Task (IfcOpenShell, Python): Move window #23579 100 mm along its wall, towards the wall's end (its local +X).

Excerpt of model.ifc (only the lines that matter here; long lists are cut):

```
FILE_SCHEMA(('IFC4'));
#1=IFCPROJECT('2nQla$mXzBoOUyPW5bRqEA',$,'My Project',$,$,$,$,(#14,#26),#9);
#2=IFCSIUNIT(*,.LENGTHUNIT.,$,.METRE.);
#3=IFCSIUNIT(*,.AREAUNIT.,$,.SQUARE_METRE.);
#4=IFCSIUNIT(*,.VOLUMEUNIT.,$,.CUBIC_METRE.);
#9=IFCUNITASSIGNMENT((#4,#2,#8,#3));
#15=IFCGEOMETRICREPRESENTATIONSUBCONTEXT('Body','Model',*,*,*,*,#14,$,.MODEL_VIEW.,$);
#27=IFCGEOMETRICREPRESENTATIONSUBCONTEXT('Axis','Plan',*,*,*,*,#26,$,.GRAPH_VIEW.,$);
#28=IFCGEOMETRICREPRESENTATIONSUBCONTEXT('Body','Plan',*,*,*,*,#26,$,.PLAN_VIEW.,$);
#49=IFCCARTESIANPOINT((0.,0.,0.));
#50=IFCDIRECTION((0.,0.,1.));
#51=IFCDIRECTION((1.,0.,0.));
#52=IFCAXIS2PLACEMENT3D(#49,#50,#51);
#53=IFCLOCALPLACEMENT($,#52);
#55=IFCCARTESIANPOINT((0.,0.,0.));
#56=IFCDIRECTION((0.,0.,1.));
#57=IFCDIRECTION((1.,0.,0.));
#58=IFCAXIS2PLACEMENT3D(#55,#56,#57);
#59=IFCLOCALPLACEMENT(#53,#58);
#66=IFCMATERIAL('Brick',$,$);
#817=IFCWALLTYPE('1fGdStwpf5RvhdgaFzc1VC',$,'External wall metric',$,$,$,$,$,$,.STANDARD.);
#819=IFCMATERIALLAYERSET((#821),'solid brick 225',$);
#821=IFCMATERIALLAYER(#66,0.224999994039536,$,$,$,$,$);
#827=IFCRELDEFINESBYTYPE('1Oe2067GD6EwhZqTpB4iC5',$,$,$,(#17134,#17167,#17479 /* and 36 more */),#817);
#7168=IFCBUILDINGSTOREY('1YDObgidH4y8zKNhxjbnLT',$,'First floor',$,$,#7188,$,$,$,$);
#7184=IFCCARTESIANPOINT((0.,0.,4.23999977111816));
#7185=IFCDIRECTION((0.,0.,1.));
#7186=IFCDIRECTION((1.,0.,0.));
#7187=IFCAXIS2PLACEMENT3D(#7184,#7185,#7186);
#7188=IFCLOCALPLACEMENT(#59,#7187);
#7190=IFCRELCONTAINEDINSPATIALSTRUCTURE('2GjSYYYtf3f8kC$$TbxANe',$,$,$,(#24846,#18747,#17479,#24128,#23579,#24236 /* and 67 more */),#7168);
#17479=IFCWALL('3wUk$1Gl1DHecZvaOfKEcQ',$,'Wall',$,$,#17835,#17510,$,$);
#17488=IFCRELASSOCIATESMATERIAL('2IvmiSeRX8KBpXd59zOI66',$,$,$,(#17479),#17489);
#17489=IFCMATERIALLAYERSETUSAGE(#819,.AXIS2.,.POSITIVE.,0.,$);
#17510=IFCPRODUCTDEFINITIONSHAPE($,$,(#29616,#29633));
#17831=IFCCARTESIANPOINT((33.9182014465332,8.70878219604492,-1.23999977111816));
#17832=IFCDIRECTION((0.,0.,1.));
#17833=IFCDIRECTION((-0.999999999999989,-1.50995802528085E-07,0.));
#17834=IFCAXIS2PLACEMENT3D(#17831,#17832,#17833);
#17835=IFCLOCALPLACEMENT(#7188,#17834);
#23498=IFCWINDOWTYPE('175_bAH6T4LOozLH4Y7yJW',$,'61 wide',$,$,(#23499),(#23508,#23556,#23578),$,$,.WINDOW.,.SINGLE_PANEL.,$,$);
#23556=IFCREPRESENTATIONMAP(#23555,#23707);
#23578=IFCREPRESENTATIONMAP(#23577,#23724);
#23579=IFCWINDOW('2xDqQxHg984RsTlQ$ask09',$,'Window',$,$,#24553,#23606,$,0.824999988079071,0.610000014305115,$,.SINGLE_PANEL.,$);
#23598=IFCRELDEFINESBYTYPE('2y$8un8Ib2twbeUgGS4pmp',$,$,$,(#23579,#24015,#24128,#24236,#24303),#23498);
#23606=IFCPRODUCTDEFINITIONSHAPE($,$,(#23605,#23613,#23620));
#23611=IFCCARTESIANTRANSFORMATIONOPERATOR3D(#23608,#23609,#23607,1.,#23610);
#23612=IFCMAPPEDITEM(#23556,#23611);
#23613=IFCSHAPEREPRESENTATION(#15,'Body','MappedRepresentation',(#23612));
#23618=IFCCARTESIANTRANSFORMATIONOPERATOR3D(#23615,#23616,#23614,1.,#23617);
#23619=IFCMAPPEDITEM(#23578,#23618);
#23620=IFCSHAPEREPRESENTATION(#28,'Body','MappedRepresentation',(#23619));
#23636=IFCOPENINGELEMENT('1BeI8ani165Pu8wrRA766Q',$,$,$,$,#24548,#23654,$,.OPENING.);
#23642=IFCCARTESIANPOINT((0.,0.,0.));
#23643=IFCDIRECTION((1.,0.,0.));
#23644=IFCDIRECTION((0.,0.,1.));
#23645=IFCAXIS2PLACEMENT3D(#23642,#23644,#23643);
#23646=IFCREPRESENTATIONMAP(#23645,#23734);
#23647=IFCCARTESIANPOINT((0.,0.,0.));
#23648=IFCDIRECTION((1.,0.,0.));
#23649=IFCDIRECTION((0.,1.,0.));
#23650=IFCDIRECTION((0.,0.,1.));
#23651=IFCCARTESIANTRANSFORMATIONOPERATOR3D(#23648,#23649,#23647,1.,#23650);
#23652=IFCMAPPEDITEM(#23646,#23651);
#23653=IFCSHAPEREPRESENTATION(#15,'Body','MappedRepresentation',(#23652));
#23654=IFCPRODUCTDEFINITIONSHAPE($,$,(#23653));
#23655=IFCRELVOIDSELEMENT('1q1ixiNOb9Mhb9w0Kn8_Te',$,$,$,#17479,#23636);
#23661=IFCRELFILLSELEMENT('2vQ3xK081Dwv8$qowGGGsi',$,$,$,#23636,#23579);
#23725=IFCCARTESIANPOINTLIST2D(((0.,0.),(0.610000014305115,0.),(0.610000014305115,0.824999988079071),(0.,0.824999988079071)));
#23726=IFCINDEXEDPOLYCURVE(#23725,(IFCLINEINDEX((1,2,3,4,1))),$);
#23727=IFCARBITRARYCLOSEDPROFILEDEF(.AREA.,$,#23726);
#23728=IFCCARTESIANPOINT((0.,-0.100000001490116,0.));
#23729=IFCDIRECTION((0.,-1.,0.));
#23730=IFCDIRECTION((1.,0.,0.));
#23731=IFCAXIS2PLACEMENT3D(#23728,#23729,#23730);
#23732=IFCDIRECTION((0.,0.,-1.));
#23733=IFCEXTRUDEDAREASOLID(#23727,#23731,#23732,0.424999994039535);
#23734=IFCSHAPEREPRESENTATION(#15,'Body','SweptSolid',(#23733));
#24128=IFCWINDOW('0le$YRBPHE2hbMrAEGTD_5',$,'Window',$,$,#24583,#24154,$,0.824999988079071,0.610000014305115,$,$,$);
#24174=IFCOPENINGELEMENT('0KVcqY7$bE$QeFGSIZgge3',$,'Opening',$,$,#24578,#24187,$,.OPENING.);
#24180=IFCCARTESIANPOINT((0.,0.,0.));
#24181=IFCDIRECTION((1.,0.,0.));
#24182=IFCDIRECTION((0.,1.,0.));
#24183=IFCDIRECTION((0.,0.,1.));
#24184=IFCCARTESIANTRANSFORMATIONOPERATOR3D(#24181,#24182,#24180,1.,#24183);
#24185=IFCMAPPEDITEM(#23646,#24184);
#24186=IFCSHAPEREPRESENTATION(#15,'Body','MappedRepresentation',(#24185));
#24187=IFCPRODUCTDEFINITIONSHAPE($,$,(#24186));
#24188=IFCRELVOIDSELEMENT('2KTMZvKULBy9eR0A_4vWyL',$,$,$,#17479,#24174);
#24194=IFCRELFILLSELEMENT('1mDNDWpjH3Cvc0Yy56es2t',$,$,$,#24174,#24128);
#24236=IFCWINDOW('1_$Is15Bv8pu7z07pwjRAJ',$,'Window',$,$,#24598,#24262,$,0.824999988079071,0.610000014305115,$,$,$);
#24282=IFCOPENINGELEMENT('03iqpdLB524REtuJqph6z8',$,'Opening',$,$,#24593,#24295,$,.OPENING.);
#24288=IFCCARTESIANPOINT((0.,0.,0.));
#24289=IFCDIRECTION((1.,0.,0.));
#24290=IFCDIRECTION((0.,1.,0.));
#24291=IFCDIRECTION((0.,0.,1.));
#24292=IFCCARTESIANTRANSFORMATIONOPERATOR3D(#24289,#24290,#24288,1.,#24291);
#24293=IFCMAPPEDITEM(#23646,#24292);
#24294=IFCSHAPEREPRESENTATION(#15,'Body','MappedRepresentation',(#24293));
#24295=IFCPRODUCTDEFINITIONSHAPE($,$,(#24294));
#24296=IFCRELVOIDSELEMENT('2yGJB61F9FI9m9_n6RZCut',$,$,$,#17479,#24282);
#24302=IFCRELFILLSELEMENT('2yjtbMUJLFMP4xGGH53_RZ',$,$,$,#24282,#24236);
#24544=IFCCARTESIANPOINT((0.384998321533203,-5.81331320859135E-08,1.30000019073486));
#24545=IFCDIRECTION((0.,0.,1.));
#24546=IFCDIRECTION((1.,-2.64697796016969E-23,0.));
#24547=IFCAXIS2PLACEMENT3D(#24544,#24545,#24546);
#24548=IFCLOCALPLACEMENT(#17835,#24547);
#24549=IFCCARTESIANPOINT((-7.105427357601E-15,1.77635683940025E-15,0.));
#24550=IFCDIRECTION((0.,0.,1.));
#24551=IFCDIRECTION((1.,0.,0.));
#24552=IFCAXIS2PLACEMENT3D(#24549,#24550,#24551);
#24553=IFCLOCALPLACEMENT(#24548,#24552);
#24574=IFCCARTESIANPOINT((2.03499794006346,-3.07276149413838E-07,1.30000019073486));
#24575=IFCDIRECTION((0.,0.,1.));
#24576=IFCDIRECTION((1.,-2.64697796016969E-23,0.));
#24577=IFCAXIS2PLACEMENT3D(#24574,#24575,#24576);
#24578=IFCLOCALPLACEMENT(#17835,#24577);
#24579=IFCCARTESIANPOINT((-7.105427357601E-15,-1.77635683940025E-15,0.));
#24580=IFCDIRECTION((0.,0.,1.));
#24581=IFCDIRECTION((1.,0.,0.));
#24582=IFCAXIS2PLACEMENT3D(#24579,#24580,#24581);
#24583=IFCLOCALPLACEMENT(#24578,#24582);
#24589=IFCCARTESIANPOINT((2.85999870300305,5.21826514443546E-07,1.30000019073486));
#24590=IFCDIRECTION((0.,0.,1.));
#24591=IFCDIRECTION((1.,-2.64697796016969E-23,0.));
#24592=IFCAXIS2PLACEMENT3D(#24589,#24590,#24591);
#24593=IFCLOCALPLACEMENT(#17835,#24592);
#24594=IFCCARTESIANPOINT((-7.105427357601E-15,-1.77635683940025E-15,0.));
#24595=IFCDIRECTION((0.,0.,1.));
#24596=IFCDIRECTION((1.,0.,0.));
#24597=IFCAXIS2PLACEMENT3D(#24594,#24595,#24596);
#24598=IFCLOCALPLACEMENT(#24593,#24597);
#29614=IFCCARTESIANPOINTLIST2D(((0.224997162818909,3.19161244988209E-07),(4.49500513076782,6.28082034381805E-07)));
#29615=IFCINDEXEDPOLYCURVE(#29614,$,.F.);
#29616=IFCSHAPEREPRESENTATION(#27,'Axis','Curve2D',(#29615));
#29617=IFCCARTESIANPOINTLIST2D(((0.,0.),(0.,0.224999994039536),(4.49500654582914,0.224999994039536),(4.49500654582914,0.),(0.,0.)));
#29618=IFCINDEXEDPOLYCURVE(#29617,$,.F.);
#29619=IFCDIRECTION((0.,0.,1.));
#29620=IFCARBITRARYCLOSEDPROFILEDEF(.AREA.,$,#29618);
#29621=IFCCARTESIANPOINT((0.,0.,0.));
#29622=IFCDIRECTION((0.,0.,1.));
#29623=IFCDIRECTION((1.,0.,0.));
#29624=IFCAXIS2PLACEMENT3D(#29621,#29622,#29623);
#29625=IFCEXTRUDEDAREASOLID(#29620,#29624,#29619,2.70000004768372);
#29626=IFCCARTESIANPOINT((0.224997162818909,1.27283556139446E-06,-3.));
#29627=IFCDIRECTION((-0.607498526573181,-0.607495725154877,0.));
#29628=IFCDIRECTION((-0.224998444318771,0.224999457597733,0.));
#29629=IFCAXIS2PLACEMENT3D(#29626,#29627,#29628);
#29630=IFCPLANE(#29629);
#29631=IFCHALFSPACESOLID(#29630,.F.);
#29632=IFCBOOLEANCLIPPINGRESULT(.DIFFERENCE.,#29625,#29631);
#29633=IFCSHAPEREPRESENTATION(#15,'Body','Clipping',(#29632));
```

```python
import ifcopenshell
import ifcopenshell.api.geometry
import ifcopenshell.util.placement

model = ifcopenshell.open("model.ifc")

window = model.by_guid("2xDqQxHg984RsTlQ$ask09")
opening = window.FillsVoids[0].RelatingOpeningElement
wall = opening.VoidsElements[0].RelatingBuildingElement

wall_matrix = ifcopenshell.util.placement.get_local_placement(wall.ObjectPlacement)
shift = wall_matrix[:3, 0] * 0.1
before = ifcopenshell.util.placement.get_local_placement(window.ObjectPlacement)[:3, 3].copy()

# The window is placed relative to its opening, so it follows when the opening moves.
matrix = ifcopenshell.util.placement.get_local_placement(opening.ObjectPlacement)
matrix[:3, 3] += shift
ifcopenshell.api.geometry.edit_object_placement(
    model, product=opening, matrix=matrix, is_si=False, should_transform_children=True
)

after = ifcopenshell.util.placement.get_local_placement(window.ObjectPlacement)[:3, 3]
print("window moved by", (after - before).round(3) + 0.0)

model.write("model_updated.ifc")
```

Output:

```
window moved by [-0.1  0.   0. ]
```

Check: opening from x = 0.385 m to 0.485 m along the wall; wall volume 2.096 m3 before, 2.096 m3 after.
